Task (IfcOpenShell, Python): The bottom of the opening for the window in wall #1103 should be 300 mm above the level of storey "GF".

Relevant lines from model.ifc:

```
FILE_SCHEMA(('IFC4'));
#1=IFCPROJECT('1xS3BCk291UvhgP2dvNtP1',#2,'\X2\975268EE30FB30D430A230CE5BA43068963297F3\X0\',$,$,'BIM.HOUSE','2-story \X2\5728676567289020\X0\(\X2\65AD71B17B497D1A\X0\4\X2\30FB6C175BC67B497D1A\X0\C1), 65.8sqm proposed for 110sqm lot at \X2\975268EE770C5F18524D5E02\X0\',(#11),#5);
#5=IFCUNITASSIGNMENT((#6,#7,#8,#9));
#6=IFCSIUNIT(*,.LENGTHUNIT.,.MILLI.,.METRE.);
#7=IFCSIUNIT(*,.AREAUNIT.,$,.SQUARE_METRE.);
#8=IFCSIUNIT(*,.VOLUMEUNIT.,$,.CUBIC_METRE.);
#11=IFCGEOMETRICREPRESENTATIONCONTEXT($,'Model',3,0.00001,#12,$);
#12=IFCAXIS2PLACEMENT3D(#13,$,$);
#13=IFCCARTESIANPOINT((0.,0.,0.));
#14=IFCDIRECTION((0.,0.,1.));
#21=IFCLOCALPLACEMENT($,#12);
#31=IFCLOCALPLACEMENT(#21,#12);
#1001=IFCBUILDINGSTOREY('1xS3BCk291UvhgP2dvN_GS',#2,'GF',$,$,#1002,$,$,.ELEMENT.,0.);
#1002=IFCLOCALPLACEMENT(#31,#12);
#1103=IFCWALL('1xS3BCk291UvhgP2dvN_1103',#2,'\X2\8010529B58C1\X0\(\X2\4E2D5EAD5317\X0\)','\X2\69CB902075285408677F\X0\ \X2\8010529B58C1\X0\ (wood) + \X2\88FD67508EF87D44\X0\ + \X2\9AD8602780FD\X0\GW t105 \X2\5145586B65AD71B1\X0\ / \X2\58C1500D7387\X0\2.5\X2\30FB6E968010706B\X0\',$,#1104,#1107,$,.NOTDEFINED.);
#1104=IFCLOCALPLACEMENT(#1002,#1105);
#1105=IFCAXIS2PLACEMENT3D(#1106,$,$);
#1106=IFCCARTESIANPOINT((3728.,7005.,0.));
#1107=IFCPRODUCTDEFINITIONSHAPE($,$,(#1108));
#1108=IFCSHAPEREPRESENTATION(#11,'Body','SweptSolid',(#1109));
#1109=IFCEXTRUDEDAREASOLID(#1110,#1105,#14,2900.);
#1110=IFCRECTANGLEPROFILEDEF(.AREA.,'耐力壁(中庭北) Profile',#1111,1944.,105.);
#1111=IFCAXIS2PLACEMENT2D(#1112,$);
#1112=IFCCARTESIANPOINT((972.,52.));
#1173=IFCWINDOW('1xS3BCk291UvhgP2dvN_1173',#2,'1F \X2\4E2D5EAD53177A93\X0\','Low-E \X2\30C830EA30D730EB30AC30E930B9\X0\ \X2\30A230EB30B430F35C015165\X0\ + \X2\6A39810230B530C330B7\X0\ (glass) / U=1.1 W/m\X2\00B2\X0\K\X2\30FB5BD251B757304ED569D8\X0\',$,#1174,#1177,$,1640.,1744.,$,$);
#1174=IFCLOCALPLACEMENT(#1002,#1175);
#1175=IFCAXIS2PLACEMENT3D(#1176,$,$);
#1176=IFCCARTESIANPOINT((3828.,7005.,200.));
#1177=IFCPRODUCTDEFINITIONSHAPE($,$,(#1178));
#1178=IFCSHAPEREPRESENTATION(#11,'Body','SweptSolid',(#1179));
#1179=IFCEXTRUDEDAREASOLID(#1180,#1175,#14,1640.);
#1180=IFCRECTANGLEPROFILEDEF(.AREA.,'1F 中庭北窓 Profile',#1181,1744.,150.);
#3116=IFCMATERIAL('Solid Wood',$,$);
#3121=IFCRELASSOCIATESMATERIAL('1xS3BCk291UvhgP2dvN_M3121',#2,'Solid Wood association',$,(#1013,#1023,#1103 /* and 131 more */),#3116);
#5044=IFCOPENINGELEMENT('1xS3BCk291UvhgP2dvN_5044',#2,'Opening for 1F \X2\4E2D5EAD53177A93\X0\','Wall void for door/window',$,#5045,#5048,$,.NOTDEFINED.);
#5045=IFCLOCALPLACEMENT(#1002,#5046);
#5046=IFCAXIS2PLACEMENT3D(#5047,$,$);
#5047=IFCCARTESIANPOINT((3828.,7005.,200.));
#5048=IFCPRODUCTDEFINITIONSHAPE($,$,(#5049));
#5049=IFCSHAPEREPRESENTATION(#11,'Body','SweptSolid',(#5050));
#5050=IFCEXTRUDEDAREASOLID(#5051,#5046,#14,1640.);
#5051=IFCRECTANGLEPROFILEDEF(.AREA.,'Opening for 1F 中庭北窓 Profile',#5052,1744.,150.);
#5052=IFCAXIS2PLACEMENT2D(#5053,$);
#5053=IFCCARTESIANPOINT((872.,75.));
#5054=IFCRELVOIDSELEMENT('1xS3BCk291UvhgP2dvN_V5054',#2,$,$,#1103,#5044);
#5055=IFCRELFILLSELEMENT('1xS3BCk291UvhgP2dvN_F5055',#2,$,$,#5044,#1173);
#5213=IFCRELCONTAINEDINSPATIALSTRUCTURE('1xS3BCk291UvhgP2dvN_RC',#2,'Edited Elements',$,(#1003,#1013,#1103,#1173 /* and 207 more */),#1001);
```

```python
import numpy as np
import ifcopenshell
import ifcopenshell.api.geometry
import ifcopenshell.geom
import ifcopenshell.util.element
import ifcopenshell.util.placement
import ifcopenshell.util.shape
import ifcopenshell.util.unit

model = ifcopenshell.open("model.ifc")
unit_scale = ifcopenshell.util.unit.calculate_unit_scale(model)

window = model.by_guid("1xS3BCk291UvhgP2dvN_1173")
opening = window.FillsVoids[0].RelatingOpeningElement
storey = ifcopenshell.util.element.get_container(window, ifc_class="IfcBuildingStorey")
level = ifcopenshell.util.placement.get_local_placement(storey.ObjectPlacement)[2, 3]

# The opening's origin need not be at the sill, so measure its lowest point.
shape = ifcopenshell.geom.create_shape(ifcopenshell.geom.settings(), opening)
bottom = ifcopenshell.util.shape.get_shape_bottom_elevation(shape, shape.geometry) / unit_scale
dz = level + 0.3 / unit_scale - bottom

shift = np.array([0.0, 0.0, dz])
# The window is not placed relative to its opening, so move both.
for product in (opening, window):
    matrix = ifcopenshell.util.placement.get_local_placement(product.ObjectPlacement)
    matrix[:3, 3] += shift
    ifcopenshell.api.geometry.edit_object_placement(model, product=product, matrix=matrix, is_si=False)

print(f"moved by {dz * unit_scale:+.3f} m")

model.write("model_edited.ifc")
```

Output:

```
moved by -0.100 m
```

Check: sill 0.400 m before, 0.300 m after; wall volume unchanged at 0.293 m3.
